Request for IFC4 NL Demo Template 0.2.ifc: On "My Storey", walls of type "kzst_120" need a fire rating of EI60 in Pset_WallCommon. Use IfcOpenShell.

First a look at what the model holds.

```python
import ifcopenshell
import ifcopenshell.util.element

model = ifcopenshell.open("IFC4 NL Demo Template 0.2.ifc")
print(model.schema)
storey = next(s for s in model.by_type("IfcBuildingStorey") if s.Name == "My Storey")
walls = [e for e in ifcopenshell.util.element.get_decomposition(storey) if e.is_a("IfcWall")]
seen = {}
for e in walls:
    element_type = ifcopenshell.util.element.get_type(e)
    key = (element_type.Name if element_type != e and element_type else None, ifcopenshell.util.element.get_pset(e, "Pset_WallCommon", "FireRating"))
    seen[key] = seen.get(key, 0) + 1
for (name, value), count in sorted(seen.items(), key=str):
    print(count, "x", name, "|", value)
```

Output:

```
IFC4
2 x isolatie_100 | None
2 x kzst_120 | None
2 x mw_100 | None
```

```python
import ifcopenshell
import ifcopenshell.api.pset
import ifcopenshell.util.element

model = ifcopenshell.open("IFC4 NL Demo Template 0.2.ifc")

storey = next(s for s in model.by_type("IfcBuildingStorey") if s.Name == "My Storey")
walls = [e for e in ifcopenshell.util.element.get_decomposition(storey) if e.is_a("IfcWall")]

count = 0
for e in walls:
    element_type = ifcopenshell.util.element.get_type(e)
    if element_type in (None, e) or element_type.Name != "kzst_120":
        continue
    # add_pset returns the element's existing set when there is one.
    pset = ifcopenshell.api.pset.add_pset(model, product=e, name="Pset_WallCommon")
    ifcopenshell.api.pset.edit_pset(model, pset=pset, properties={"FireRating": "EI60"})
    count += 1

print(count, "walls updated")

model.write("IFC4 NL Demo Template 0.2_rev.ifc")
```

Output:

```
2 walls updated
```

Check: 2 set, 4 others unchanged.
